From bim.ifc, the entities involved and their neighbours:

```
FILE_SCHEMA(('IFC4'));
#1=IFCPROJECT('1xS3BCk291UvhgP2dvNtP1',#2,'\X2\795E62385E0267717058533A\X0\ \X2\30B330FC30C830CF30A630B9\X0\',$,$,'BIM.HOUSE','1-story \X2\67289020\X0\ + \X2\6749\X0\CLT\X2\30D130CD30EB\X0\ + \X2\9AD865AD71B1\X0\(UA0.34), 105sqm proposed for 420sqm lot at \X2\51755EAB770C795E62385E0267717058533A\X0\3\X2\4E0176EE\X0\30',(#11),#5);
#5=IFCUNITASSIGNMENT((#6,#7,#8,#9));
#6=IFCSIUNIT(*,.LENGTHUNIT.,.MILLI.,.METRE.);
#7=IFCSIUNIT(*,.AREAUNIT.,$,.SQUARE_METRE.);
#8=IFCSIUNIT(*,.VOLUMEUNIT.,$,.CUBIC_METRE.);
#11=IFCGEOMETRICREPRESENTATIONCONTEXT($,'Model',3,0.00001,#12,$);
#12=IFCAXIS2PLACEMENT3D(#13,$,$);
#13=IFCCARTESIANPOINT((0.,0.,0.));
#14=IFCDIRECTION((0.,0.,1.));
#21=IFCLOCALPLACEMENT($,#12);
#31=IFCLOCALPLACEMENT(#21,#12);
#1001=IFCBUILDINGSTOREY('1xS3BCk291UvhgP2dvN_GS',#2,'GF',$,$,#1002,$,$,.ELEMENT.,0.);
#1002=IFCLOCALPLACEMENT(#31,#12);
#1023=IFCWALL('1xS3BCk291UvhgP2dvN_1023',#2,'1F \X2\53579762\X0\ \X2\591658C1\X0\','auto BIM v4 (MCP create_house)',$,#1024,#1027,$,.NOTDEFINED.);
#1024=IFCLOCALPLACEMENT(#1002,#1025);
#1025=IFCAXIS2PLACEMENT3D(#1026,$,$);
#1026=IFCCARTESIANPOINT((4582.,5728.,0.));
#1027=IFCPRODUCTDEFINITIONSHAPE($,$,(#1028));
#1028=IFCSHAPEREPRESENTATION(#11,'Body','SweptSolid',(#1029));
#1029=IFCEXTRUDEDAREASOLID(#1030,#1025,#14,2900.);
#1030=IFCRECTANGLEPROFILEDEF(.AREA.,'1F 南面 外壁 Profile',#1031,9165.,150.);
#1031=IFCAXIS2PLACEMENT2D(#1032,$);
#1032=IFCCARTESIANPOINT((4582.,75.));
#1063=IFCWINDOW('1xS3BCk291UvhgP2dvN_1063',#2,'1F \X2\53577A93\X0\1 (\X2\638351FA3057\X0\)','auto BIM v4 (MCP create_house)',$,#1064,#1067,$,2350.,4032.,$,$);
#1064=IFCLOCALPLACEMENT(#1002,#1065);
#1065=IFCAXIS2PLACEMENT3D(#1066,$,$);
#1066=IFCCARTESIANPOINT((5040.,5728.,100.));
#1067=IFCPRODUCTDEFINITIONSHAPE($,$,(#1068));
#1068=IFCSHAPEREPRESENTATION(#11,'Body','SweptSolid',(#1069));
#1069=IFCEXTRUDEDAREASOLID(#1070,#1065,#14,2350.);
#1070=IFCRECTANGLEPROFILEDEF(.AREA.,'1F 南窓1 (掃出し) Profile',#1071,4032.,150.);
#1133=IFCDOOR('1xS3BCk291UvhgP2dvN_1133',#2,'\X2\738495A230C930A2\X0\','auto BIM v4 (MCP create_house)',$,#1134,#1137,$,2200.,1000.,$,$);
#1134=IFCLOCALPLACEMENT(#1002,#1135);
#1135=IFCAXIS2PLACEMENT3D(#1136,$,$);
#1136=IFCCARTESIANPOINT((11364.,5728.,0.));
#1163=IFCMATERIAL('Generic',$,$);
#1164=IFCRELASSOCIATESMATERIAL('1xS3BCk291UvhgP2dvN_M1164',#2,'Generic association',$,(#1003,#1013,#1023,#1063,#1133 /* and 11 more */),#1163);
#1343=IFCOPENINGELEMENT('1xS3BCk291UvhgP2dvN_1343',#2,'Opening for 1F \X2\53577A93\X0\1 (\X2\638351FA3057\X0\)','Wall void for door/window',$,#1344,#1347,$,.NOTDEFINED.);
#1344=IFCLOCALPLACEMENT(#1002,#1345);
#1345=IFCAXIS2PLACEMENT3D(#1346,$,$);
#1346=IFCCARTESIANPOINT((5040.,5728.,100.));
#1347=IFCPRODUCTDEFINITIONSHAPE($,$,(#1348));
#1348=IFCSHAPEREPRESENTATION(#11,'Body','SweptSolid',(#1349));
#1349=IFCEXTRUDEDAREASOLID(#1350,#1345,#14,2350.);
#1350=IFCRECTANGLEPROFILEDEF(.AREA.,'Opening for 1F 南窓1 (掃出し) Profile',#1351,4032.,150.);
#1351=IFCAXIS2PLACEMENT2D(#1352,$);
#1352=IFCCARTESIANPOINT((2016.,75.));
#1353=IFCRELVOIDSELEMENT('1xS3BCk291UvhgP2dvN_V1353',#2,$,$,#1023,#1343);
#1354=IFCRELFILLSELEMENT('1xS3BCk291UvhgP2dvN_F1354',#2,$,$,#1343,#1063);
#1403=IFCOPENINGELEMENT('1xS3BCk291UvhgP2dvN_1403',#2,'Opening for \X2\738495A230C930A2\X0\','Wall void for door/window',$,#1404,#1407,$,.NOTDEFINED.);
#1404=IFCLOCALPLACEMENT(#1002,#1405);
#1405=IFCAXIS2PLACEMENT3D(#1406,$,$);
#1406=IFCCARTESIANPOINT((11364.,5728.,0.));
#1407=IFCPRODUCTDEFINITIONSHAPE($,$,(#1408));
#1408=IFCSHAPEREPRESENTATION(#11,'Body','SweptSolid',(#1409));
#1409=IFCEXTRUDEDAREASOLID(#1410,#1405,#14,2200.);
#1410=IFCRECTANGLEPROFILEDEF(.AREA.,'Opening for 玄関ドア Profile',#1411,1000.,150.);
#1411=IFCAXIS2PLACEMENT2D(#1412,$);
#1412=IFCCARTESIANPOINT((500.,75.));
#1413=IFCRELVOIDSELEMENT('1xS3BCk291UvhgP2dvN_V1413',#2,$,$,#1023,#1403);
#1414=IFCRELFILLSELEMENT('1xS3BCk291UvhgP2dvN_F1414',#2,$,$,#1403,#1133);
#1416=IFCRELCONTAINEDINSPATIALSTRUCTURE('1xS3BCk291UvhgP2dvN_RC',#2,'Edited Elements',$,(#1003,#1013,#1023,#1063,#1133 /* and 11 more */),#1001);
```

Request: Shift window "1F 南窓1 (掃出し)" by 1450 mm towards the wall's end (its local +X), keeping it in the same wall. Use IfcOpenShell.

```python
import ifcopenshell
import ifcopenshell.api.geometry
import ifcopenshell.util.placement
import ifcopenshell.util.unit

model = ifcopenshell.open("bim.ifc")
unit_scale = ifcopenshell.util.unit.calculate_unit_scale(model)

window = model.by_guid("1xS3BCk291UvhgP2dvN_1063")
opening = window.FillsVoids[0].RelatingOpeningElement
wall = opening.VoidsElements[0].RelatingBuildingElement

wall_matrix = ifcopenshell.util.placement.get_local_placement(wall.ObjectPlacement)
shift = wall_matrix[:3, 0] * 1.45 / unit_scale
before = ifcopenshell.util.placement.get_local_placement(window.ObjectPlacement)[:3, 3].copy()

# The window is not placed relative to its opening, so move both.
for product in (opening, window):
    matrix = ifcopenshell.util.placement.get_local_placement(product.ObjectPlacement)
    matrix[:3, 3] += shift
    ifcopenshell.api.geometry.edit_object_placement(model, product=product, matrix=matrix, is_si=False)

after = ifcopenshell.util.placement.get_local_placement(window.ObjectPlacement)[:3, 3]
print("window moved by", (after - before).round(3) + 0.0)

model.write("bim_v2.ifc")
```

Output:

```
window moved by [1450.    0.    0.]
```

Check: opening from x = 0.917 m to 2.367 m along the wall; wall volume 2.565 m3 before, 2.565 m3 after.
